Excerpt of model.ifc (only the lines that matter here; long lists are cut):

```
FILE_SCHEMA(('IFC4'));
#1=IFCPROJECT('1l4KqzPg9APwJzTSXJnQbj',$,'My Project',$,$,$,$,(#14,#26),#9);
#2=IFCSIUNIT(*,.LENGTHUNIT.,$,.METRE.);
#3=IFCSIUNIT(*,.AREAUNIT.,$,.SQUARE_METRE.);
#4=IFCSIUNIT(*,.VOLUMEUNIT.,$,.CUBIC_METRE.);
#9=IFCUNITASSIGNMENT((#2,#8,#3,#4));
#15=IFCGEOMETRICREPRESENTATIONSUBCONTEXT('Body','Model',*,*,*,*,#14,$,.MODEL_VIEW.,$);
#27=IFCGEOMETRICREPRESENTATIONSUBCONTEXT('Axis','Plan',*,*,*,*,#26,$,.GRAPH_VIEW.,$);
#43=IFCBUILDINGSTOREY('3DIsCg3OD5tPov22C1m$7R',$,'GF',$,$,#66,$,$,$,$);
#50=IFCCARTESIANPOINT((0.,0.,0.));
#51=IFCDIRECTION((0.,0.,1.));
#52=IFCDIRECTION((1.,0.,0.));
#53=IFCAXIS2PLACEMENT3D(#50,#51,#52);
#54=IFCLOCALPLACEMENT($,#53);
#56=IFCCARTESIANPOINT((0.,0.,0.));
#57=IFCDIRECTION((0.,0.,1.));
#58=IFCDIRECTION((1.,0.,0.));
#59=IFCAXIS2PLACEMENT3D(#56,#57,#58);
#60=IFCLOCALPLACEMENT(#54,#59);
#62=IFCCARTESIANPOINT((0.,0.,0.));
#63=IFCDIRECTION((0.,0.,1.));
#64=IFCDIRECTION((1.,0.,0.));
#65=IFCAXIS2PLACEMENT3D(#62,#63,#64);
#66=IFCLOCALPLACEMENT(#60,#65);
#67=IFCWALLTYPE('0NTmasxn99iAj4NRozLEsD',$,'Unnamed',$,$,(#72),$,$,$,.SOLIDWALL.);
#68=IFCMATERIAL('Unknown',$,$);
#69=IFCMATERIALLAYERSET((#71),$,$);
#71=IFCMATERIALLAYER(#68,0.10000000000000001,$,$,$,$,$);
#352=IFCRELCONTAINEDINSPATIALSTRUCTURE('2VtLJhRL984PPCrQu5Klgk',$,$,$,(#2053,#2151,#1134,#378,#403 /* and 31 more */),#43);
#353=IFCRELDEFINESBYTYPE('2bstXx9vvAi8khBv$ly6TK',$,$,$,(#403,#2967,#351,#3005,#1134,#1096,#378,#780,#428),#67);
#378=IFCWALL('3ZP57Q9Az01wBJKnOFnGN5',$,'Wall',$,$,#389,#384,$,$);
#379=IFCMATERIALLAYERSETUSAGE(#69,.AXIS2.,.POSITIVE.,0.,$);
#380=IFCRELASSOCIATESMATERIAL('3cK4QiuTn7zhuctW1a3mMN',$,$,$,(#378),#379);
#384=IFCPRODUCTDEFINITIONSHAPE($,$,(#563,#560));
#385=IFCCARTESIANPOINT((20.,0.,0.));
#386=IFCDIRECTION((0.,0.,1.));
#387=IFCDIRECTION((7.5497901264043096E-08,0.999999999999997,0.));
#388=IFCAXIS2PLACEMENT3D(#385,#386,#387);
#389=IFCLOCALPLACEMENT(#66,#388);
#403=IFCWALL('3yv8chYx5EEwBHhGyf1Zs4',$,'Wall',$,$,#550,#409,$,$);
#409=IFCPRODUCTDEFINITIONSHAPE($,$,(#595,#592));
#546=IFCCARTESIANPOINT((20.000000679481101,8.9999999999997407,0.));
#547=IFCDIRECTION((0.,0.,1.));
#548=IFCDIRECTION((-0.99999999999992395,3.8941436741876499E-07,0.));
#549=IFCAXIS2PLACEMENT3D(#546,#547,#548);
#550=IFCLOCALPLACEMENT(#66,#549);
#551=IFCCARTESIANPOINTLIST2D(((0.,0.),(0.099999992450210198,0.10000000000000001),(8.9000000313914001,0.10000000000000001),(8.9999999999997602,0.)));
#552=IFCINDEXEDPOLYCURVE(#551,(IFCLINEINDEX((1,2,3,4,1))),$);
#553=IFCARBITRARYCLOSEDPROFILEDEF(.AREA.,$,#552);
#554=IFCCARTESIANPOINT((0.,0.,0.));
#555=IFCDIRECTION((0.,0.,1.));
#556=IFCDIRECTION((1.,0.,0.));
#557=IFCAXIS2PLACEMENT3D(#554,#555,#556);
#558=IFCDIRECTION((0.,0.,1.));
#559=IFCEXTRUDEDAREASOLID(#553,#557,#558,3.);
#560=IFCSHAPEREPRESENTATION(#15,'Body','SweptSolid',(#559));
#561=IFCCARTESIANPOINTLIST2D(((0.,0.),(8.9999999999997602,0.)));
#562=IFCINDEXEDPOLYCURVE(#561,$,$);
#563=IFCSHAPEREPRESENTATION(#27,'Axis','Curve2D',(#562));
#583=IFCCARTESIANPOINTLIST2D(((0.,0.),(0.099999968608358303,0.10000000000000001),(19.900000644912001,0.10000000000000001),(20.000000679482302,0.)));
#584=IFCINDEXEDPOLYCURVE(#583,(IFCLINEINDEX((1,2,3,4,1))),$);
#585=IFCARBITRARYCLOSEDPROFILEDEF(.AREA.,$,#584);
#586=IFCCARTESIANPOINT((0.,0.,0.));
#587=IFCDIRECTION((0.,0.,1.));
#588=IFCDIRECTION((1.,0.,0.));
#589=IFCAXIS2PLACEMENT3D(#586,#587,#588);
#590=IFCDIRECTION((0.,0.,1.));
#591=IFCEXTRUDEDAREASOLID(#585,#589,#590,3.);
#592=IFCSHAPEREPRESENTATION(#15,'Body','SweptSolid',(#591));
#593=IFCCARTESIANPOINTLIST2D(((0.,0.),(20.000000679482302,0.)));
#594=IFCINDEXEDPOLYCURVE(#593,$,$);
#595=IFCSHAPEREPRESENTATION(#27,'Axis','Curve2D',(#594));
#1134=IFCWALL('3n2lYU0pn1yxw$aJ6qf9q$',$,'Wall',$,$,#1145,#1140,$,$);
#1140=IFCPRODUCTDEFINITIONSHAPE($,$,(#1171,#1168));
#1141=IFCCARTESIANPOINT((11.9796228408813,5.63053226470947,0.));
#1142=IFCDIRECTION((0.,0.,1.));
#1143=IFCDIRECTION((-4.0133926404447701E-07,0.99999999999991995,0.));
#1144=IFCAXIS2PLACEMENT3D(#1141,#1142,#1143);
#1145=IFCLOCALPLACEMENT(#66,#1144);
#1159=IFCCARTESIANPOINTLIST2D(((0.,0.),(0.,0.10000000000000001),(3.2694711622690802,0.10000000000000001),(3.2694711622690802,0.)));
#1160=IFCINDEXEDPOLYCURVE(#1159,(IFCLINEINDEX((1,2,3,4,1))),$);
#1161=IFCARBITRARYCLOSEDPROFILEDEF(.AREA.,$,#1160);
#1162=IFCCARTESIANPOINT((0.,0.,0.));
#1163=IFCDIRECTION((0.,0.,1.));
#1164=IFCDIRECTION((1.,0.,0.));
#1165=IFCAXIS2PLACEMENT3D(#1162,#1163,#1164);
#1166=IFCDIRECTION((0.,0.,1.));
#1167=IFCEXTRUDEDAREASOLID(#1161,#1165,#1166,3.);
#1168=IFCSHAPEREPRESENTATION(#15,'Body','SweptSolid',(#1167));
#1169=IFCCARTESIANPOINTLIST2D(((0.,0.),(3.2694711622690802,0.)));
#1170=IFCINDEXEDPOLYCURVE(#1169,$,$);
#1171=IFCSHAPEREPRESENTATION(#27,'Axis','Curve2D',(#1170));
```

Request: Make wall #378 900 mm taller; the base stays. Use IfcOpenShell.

```python
import ifcopenshell
import ifcopenshell.geom
import ifcopenshell.util.representation
import ifcopenshell.util.shape
import ifcopenshell.util.unit

model = ifcopenshell.open("model.ifc")
unit_scale = ifcopenshell.util.unit.calculate_unit_scale(model)
settings = ifcopenshell.geom.settings()


def volume(element):
    """Net volume in cubic metres, openings subtracted."""
    shape = ifcopenshell.geom.create_shape(settings, element)
    return ifcopenshell.util.shape.get_volume(shape.geometry)


wall = model.by_guid("3ZP57Q9Az01wBJKnOFnGN5")
before = volume(wall)

body = ifcopenshell.util.representation.get_representation(wall, "Model", "Body")
solid = body.Items[0]
old_height = solid.Depth
solid.Depth += 0.9 / unit_scale
after = volume(wall)

print(f"height {old_height:g} -> {solid.Depth:g}, volume {before:.3f} -> {after:.3f} m3")

model.write("model_v2.ifc")
```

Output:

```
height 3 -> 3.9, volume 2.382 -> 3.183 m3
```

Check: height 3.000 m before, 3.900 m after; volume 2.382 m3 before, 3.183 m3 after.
